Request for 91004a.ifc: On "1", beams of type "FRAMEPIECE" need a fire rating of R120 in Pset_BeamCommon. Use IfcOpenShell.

First a look at what the model holds.

```python
import ifcopenshell
import ifcopenshell.util.element

model = ifcopenshell.open("91004a.ifc")
print(model.schema)
storey = next(s for s in model.by_type("IfcBuildingStorey") if s.Name == "1")
beams = [e for e in ifcopenshell.util.element.get_decomposition(storey) if e.is_a("IfcBeam")]
seen = {}
for e in beams:
    element_type = ifcopenshell.util.element.get_type(e)
    key = (element_type.Name if element_type != e and element_type else None, ifcopenshell.util.element.get_pset(e, "Pset_BeamCommon", "FireRating"))
    seen[key] = seen.get(key, 0) + 1
for (name, value), count in sorted(seen.items(), key=str):
    print(count, "x", name, "|", value)
```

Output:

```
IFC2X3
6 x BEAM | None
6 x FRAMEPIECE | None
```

```python
import ifcopenshell
import ifcopenshell.api.pset
import ifcopenshell.util.element

model = ifcopenshell.open("91004a.ifc")

storey = next(s for s in model.by_type("IfcBuildingStorey") if s.Name == "1")
beams = [e for e in ifcopenshell.util.element.get_decomposition(storey) if e.is_a("IfcBeam")]

count = 0
for e in beams:
    element_type = ifcopenshell.util.element.get_type(e)
    if element_type in (None, e) or element_type.Name != "FRAMEPIECE":
        continue
    # add_pset returns the element's existing set when there is one.
    pset = ifcopenshell.api.pset.add_pset(model, product=e, name="Pset_BeamCommon")
    ifcopenshell.api.pset.edit_pset(model, pset=pset, properties={"FireRating": "R120"})
    count += 1

print(count, "beams updated")

model.write("91004a-out.ifc")
```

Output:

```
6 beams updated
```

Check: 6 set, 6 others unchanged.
